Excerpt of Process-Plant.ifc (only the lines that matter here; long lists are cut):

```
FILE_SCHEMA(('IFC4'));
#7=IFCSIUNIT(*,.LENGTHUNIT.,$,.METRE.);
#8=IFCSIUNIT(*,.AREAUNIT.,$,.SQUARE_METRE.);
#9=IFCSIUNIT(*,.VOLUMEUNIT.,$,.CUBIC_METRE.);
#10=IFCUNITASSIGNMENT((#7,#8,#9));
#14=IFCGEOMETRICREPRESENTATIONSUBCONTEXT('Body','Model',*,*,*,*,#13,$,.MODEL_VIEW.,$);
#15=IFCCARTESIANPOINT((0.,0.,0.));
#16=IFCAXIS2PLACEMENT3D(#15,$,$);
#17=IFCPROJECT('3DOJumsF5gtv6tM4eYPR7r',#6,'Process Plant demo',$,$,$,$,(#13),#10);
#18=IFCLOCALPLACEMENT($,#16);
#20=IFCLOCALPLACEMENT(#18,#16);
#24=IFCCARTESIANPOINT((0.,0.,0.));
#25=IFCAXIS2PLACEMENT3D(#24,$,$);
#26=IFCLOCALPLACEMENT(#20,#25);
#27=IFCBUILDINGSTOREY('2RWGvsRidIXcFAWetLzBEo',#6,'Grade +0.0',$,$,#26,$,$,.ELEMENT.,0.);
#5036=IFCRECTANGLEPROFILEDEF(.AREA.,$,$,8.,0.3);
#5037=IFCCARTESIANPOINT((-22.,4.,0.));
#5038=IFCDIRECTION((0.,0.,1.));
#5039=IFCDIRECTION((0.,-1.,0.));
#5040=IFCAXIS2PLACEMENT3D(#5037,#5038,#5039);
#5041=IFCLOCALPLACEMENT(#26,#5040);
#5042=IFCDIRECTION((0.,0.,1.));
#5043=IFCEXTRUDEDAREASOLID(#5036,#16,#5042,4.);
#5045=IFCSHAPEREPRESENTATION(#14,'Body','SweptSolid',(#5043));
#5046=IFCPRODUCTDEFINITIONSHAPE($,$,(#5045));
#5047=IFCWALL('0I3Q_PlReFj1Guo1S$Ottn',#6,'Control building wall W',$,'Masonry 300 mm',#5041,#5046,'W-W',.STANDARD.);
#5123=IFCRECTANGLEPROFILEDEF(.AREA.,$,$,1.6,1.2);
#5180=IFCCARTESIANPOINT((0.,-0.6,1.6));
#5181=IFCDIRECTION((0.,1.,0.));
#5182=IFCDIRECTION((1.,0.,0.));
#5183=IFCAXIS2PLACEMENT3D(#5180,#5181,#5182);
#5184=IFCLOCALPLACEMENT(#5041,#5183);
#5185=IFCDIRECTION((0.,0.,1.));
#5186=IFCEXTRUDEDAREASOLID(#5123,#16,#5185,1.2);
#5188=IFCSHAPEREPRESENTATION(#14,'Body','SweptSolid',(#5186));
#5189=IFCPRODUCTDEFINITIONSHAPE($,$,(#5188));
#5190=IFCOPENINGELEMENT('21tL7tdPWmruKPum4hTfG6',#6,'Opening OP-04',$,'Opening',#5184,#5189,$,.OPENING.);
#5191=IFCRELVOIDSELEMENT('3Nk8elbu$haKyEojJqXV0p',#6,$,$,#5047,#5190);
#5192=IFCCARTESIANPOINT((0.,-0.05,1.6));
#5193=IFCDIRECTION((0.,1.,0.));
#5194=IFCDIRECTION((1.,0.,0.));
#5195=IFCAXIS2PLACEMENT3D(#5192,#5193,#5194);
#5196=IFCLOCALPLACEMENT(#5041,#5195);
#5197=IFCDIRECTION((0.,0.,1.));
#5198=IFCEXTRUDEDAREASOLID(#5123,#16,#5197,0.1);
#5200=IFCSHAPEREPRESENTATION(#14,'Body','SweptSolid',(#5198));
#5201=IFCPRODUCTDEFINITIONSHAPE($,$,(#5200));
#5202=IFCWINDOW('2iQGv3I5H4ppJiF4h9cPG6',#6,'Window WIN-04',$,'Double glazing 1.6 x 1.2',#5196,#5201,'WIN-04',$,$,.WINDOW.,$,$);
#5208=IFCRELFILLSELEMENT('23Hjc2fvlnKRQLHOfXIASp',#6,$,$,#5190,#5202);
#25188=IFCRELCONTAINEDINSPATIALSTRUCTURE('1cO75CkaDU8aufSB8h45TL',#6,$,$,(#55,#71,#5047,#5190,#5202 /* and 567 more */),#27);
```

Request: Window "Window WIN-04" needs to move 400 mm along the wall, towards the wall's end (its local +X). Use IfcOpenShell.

```python
import ifcopenshell
import ifcopenshell.api.geometry
import ifcopenshell.util.placement

model = ifcopenshell.open("Process-Plant.ifc")

window = model.by_id(5202)
opening = window.FillsVoids[0].RelatingOpeningElement
wall = opening.VoidsElements[0].RelatingBuildingElement

wall_matrix = ifcopenshell.util.placement.get_local_placement(wall.ObjectPlacement)
shift = wall_matrix[:3, 0] * 0.4
before = ifcopenshell.util.placement.get_local_placement(window.ObjectPlacement)[:3, 3].copy()

# The window is not placed relative to its opening, so move both.
for product in (opening, window):
    matrix = ifcopenshell.util.placement.get_local_placement(product.ObjectPlacement)
    matrix[:3, 3] += shift
    ifcopenshell.api.geometry.edit_object_placement(model, product=product, matrix=matrix, is_si=False)

after = ifcopenshell.util.placement.get_local_placement(window.ObjectPlacement)[:3, 3]
print("window moved by", (after - before).round(3) + 0.0)

model.write("Process-Plant_edited.ifc")
```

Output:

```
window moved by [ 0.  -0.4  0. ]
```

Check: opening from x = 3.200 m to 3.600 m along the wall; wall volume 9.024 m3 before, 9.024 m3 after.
